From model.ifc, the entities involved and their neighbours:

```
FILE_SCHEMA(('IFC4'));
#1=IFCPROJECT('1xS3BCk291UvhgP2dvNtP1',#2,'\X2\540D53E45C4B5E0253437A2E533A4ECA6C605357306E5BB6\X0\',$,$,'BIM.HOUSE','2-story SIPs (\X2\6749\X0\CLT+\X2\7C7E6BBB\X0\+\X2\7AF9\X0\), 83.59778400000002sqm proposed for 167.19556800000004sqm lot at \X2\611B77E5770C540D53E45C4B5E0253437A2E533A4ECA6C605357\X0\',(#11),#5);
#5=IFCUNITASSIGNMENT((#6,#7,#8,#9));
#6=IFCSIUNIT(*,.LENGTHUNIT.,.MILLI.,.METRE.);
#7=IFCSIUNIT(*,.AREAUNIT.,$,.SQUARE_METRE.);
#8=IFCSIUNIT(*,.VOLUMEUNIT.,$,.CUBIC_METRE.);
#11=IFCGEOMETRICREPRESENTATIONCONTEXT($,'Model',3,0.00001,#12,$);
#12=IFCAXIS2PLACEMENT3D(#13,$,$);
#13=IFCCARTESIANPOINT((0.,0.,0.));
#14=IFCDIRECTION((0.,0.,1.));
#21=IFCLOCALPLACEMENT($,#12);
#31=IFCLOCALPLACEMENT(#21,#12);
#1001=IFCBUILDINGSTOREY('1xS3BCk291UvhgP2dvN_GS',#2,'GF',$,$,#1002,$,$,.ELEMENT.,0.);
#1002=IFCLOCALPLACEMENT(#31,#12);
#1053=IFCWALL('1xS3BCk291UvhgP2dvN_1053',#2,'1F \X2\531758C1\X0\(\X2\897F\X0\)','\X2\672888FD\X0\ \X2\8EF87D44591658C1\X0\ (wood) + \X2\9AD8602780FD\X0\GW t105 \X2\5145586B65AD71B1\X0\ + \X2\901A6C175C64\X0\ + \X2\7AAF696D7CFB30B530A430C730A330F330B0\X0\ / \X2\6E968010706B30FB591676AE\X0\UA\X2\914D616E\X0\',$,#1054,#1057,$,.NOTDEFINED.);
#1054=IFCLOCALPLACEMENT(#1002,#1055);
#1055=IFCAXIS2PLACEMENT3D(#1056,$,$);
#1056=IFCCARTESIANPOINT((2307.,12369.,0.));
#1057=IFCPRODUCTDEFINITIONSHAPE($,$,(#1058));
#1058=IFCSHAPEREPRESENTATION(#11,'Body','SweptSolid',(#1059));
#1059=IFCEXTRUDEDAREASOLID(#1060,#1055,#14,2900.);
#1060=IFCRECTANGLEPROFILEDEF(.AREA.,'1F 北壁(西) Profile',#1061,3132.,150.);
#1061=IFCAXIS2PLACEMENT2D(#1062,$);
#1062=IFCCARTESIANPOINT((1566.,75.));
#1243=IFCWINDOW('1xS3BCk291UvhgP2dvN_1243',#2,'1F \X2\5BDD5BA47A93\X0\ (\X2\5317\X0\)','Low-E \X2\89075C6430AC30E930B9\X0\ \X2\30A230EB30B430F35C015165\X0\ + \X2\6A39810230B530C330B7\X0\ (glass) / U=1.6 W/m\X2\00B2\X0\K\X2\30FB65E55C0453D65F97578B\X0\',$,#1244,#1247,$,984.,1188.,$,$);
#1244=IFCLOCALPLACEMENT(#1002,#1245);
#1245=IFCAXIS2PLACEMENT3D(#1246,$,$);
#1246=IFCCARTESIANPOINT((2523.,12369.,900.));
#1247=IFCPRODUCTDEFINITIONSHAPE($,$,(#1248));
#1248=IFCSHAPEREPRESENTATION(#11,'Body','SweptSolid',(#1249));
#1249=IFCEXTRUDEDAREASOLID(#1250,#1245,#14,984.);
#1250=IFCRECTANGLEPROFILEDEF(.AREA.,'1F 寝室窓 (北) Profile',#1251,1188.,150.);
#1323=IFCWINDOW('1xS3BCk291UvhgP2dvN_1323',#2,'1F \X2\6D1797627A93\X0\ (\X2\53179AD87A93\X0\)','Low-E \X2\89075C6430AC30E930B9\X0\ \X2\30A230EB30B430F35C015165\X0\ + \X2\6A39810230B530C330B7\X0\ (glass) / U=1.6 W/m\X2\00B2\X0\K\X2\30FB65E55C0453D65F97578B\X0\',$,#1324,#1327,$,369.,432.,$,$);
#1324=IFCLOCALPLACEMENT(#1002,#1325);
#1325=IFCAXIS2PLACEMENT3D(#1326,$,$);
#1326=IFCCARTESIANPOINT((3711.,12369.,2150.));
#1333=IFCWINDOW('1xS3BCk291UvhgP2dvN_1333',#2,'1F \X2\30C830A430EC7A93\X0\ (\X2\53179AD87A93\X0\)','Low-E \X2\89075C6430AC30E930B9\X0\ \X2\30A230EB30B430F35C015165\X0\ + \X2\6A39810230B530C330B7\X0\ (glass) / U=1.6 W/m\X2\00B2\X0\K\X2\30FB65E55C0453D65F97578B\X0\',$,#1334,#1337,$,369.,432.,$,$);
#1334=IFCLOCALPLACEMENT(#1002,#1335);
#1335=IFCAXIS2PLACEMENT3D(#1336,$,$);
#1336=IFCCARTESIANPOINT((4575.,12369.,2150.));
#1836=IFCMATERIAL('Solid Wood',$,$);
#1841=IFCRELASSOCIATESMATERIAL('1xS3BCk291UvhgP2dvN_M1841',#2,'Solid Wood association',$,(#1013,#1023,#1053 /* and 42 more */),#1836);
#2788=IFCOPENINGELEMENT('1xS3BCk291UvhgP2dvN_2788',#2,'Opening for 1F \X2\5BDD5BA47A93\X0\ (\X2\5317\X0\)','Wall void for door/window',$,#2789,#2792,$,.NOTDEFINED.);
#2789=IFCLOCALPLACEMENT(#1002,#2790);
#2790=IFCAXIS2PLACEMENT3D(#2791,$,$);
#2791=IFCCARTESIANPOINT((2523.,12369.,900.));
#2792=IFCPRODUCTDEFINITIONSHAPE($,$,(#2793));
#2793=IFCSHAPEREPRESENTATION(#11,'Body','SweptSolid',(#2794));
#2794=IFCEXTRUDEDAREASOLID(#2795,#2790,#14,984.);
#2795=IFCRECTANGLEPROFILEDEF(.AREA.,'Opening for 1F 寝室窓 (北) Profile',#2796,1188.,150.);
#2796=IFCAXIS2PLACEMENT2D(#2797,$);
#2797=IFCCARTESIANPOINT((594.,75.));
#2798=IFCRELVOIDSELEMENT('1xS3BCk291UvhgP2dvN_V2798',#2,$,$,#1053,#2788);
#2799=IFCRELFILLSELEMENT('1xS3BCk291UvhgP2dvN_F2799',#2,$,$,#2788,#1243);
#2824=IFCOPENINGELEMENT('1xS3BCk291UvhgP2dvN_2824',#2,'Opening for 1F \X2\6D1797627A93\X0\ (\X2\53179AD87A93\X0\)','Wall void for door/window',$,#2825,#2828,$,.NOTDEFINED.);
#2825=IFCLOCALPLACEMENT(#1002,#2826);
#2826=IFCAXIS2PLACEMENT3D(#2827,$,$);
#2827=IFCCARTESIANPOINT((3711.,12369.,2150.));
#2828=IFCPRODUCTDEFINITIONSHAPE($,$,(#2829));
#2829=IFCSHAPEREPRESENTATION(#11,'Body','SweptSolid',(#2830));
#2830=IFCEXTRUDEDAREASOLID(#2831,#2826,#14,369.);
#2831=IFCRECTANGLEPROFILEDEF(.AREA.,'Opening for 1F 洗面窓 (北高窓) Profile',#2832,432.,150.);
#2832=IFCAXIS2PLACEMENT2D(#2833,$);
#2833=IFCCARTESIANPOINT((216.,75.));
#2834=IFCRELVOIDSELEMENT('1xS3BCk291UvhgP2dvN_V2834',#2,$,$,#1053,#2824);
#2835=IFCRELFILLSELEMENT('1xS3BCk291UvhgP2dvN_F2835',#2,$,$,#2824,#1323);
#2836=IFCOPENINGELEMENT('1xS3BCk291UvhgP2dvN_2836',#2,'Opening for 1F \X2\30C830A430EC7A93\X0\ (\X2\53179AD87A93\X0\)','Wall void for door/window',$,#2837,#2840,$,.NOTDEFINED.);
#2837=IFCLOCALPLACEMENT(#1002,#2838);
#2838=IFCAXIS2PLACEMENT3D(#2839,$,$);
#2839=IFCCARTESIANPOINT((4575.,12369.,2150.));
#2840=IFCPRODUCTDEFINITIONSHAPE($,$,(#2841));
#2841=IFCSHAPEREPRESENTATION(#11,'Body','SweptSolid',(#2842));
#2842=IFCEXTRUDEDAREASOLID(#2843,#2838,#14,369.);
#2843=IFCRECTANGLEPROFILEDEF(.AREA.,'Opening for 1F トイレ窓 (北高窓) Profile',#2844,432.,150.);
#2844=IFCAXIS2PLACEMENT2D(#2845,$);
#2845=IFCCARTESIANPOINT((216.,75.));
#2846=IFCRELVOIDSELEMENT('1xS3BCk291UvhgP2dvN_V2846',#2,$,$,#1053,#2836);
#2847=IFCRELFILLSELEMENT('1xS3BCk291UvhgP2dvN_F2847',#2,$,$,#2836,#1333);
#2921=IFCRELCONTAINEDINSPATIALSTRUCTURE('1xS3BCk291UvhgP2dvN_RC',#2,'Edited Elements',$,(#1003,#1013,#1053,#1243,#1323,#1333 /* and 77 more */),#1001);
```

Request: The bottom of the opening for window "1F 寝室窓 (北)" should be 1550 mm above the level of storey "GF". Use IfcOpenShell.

```python
import numpy as np
import ifcopenshell
import ifcopenshell.api.geometry
import ifcopenshell.geom
import ifcopenshell.util.element
import ifcopenshell.util.placement
import ifcopenshell.util.shape
import ifcopenshell.util.unit

model = ifcopenshell.open("model.ifc")
unit_scale = ifcopenshell.util.unit.calculate_unit_scale(model)

window = model.by_guid("1xS3BCk291UvhgP2dvN_1243")
opening = window.FillsVoids[0].RelatingOpeningElement
storey = ifcopenshell.util.element.get_container(window, ifc_class="IfcBuildingStorey")
level = ifcopenshell.util.placement.get_local_placement(storey.ObjectPlacement)[2, 3]

# The opening's origin need not be at the sill, so measure its lowest point.
shape = ifcopenshell.geom.create_shape(ifcopenshell.geom.settings(), opening)
bottom = ifcopenshell.util.shape.get_shape_bottom_elevation(shape, shape.geometry) / unit_scale
dz = level + 1.55 / unit_scale - bottom

shift = np.array([0.0, 0.0, dz])
# The window is not placed relative to its opening, so move both.
for product in (opening, window):
    matrix = ifcopenshell.util.placement.get_local_placement(product.ObjectPlacement)
    matrix[:3, 3] += shift
    ifcopenshell.api.geometry.edit_object_placement(model, product=product, matrix=matrix, is_si=False)

print(f"moved by {dz * unit_scale:+.3f} m")

model.write("model_updated.ifc")
```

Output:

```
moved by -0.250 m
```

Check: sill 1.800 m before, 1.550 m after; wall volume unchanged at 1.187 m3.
